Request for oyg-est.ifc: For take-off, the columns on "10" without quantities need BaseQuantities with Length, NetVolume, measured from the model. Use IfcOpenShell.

First a look at what the model holds.

```python
import ifcopenshell
import ifcopenshell.util.element
import ifcopenshell.util.unit

model = ifcopenshell.open("oyg-est.ifc")
print(model.schema)
for unit_type in ("LENGTHUNIT", "AREAUNIT", "VOLUMEUNIT"):
    print(unit_type, ifcopenshell.util.unit.calculate_unit_scale(model, unit_type))
storey = next(s for s in model.by_type("IfcBuildingStorey") if s.Name == "10")
columns = [e for e in ifcopenshell.util.element.get_decomposition(storey) if e.is_a("IfcColumn")]
for e in sorted(columns, key=lambda e: e.id()):
    print(e.id(), e.is_a(), e.Name, list(ifcopenshell.util.element.get_psets(e, qtos_only=True)), sep=" | ")
```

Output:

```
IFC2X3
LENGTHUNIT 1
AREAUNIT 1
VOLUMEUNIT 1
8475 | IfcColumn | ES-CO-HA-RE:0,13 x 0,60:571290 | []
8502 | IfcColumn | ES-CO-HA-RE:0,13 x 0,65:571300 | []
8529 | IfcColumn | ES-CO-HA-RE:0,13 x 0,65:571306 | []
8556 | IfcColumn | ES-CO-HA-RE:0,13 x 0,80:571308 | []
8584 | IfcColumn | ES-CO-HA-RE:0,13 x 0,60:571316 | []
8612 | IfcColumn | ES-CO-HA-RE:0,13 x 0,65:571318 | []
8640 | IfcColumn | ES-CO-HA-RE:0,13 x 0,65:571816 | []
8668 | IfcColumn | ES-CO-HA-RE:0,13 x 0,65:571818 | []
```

```python
import ifcopenshell
import ifcopenshell.api.pset
import ifcopenshell.geom
import ifcopenshell.util.element
import ifcopenshell.util.shape
import ifcopenshell.util.unit

model = ifcopenshell.open("oyg-est.ifc")
unit_scale = ifcopenshell.util.unit.calculate_unit_scale(model)
volume_scale = ifcopenshell.util.unit.calculate_unit_scale(model, "VOLUMEUNIT")
settings = ifcopenshell.geom.settings()

storey = next(s for s in model.by_type("IfcBuildingStorey") if s.Name == "10")
columns = [e for e in ifcopenshell.util.element.get_decomposition(storey) if e.is_a("IfcColumn")]

for e in sorted(columns, key=lambda e: e.id()):
    if ifcopenshell.util.element.get_psets(e, qtos_only=True, should_inherit=False):
        continue
    # Geometry comes back in metres, in the element's own axes.
    shape = ifcopenshell.geom.create_shape(settings, e)
    values = {
        "Length": ifcopenshell.util.shape.get_z(shape.geometry) / unit_scale,
        "NetVolume": ifcopenshell.util.shape.get_volume(shape.geometry) / volume_scale,
    }
    qto = ifcopenshell.api.pset.add_qto(model, product=e, name="BaseQuantities")
    ifcopenshell.api.pset.edit_qto(model, qto=qto, properties=values)
    print(e.id(), {k: round(v, 3) for k, v in values.items()})

model.write("oyg-est_updated.ifc")
```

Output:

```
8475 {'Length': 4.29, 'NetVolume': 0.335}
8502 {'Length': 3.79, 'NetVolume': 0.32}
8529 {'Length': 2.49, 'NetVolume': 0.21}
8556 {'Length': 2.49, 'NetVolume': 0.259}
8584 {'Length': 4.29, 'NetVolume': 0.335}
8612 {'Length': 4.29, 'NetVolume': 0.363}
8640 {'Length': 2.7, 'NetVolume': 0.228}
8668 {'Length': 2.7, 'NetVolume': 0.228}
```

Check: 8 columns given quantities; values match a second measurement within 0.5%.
